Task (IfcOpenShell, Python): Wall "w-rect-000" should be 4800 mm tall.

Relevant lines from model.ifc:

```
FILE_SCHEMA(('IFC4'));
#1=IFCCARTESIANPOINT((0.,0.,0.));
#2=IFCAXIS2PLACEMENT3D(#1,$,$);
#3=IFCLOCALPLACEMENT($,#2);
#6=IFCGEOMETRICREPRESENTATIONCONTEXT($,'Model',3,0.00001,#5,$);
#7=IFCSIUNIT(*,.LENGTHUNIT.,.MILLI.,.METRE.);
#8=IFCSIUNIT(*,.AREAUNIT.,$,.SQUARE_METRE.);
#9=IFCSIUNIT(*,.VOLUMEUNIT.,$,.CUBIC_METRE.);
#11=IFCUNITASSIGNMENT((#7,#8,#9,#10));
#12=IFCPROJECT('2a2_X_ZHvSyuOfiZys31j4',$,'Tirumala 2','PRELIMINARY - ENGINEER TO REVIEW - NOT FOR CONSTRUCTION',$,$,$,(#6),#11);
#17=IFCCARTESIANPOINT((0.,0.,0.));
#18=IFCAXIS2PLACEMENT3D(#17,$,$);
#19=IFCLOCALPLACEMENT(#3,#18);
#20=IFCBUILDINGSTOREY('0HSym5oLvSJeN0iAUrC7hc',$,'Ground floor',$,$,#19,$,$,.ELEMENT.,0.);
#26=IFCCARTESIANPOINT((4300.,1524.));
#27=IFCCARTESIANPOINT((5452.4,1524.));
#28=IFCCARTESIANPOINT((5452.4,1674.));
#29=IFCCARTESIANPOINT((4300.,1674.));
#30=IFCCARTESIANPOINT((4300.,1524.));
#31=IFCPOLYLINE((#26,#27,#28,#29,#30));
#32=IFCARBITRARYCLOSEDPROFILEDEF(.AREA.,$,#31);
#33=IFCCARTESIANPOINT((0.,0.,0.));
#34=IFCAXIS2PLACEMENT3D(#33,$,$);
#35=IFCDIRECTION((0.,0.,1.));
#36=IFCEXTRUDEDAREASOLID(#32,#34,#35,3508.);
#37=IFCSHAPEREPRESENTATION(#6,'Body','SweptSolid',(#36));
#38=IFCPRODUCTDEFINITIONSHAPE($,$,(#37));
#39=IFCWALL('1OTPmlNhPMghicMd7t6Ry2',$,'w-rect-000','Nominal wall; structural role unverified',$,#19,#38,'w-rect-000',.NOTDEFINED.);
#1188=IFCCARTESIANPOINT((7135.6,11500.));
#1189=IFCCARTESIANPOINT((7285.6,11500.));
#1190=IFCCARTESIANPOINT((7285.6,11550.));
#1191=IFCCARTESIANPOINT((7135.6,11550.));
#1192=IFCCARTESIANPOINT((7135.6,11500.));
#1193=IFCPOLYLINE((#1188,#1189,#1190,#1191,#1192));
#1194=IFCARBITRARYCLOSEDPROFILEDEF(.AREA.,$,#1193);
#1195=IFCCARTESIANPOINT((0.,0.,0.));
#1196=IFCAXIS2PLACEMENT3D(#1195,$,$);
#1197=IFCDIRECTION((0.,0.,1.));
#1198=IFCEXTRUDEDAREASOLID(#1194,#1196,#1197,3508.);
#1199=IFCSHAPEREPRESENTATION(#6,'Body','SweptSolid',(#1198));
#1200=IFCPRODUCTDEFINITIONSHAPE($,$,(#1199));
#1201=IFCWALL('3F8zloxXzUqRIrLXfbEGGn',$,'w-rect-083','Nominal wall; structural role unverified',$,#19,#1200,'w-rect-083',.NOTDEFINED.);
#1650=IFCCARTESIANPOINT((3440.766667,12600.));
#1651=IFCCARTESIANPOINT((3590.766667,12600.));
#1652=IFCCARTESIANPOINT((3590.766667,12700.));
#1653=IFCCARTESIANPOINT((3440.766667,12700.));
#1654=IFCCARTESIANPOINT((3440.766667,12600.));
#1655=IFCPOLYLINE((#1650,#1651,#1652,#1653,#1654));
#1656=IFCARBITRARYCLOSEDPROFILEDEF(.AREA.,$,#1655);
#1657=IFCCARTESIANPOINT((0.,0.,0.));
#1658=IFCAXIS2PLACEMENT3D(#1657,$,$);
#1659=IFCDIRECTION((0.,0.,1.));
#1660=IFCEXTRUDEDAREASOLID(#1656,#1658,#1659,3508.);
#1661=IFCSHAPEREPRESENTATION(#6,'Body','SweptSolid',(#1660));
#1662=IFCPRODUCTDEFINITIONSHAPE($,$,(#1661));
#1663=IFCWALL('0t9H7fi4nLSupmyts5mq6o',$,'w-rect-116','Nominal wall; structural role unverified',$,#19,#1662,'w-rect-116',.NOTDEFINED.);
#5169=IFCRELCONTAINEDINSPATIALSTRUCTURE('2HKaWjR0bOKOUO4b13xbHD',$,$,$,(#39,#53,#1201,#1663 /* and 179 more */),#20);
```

```python
import ifcopenshell
import ifcopenshell.geom
import ifcopenshell.util.shape

model = ifcopenshell.open("model.ifc")
settings = ifcopenshell.geom.settings()


def volume(element):
    """Net volume in cubic metres, openings subtracted."""
    shape = ifcopenshell.geom.create_shape(settings, element)
    return ifcopenshell.util.shape.get_volume(shape.geometry)


wall = model.by_guid("1OTPmlNhPMghicMd7t6Ry2")
before = volume(wall)

body = next(r for r in wall.Representation.Representations if r.RepresentationIdentifier == "Body")
solid = body.Items[0]
old_height = solid.Depth
solid.Depth = 4800.0
after = volume(wall)

print(f"height {old_height:g} -> {solid.Depth:g}, volume {before:.3f} -> {after:.3f} m3")

model.write("model_v2.ifc")
```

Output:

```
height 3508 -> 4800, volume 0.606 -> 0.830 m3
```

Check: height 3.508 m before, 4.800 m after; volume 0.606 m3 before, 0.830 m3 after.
